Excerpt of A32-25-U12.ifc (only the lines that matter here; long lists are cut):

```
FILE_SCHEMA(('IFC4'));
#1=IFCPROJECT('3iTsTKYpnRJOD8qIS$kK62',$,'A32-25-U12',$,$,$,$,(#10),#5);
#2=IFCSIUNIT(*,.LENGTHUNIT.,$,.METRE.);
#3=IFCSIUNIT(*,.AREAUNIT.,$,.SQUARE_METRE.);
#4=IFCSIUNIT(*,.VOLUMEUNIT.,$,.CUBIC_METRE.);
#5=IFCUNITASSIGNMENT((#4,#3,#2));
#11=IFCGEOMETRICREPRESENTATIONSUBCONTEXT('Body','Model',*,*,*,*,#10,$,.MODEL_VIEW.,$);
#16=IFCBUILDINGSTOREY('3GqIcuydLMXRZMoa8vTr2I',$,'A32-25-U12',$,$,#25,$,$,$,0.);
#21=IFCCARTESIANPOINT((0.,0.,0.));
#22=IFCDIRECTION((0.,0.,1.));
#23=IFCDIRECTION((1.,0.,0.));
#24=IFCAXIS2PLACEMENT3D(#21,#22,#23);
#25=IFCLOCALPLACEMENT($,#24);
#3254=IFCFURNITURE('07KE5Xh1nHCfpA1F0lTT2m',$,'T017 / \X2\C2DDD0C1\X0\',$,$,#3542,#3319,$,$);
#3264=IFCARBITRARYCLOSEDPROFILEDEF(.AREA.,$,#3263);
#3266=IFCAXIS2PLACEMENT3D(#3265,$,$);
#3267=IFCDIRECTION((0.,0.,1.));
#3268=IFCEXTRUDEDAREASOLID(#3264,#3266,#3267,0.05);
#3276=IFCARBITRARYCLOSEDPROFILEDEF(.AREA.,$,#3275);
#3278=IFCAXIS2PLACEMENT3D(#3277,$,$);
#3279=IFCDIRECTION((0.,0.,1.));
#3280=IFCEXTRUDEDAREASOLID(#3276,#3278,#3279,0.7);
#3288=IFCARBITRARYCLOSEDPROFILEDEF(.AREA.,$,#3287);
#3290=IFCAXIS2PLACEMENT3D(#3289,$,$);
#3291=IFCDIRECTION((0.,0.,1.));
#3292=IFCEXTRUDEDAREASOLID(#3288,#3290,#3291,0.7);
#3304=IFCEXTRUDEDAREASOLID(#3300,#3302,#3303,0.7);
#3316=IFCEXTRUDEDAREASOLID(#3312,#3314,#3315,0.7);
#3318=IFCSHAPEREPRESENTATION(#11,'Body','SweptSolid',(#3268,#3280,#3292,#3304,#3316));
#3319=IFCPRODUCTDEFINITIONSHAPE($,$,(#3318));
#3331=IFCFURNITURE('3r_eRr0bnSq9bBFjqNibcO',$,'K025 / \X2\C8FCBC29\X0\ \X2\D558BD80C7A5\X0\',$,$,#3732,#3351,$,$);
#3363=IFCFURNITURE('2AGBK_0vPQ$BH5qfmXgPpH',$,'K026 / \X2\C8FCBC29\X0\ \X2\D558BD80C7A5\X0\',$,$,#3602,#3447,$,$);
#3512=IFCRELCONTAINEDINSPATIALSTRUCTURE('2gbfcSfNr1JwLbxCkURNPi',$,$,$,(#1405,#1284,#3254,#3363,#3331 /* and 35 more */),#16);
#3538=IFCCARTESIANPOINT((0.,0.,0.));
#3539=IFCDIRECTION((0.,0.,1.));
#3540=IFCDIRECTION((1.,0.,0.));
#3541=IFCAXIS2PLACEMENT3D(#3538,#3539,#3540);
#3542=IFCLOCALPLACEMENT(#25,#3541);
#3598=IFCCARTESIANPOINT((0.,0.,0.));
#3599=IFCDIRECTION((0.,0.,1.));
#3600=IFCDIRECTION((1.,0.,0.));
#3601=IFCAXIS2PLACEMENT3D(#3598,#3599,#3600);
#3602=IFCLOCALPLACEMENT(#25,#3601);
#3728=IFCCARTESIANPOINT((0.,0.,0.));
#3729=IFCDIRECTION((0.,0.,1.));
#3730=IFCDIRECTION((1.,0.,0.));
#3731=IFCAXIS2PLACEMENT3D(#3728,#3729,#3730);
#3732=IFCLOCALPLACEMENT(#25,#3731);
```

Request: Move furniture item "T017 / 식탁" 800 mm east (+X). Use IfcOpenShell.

```python
import ifcopenshell
import ifcopenshell.api.geometry
import ifcopenshell.util.placement
import ifcopenshell.util.unit

model = ifcopenshell.open("A32-25-U12.ifc")
unit_scale = ifcopenshell.util.unit.calculate_unit_scale(model)

item = model.by_guid("07KE5Xh1nHCfpA1F0lTT2m")
matrix = ifcopenshell.util.placement.get_local_placement(item.ObjectPlacement)
matrix[0, 3] += 0.8 / unit_scale
ifcopenshell.api.geometry.edit_object_placement(model, product=item, matrix=matrix, is_si=False)

print(ifcopenshell.util.placement.get_local_placement(item.ObjectPlacement).round(3) + 0.0)

model.write("A32-25-U12_rev.ifc")
```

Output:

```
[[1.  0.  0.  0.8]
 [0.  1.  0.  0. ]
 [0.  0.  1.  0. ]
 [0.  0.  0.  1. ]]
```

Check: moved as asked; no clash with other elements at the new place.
